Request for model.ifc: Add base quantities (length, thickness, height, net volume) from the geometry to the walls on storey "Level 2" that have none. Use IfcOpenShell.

First a look at what the model holds.

```python
import ifcopenshell
import ifcopenshell.util.element
import ifcopenshell.util.unit

model = ifcopenshell.open("model.ifc")
print(model.schema)
for unit_type in ("LENGTHUNIT", "AREAUNIT", "VOLUMEUNIT"):
    print(unit_type, ifcopenshell.util.unit.calculate_unit_scale(model, unit_type))
storey = next(s for s in model.by_type("IfcBuildingStorey") if s.Name == "Level 2")
walls = [e for e in ifcopenshell.util.element.get_decomposition(storey) if e.is_a("IfcWall")]
for e in sorted(walls, key=lambda e: e.id()):
    print(e.id(), e.is_a(), e.Name, list(ifcopenshell.util.element.get_psets(e, qtos_only=True)), sep=" | ")
```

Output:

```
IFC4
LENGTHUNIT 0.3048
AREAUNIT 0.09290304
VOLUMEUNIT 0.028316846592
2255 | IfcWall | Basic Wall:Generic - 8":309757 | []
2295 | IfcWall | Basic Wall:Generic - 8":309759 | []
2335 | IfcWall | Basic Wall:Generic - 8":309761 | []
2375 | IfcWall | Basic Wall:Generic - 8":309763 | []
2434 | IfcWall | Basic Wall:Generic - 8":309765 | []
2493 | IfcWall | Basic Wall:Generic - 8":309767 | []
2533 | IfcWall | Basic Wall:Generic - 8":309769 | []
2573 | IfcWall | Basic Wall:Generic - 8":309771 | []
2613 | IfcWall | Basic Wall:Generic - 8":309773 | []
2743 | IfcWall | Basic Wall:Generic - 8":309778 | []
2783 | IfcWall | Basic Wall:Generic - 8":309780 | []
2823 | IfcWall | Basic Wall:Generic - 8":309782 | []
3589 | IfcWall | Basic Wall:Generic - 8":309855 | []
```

```python
import ifcopenshell
import ifcopenshell.api.pset
import ifcopenshell.geom
import ifcopenshell.util.element
import ifcopenshell.util.shape
import ifcopenshell.util.unit

model = ifcopenshell.open("model.ifc")
unit_scale = ifcopenshell.util.unit.calculate_unit_scale(model)
volume_scale = ifcopenshell.util.unit.calculate_unit_scale(model, "VOLUMEUNIT")
settings = ifcopenshell.geom.settings()

storey = next(s for s in model.by_type("IfcBuildingStorey") if s.Name == "Level 2")
walls = [e for e in ifcopenshell.util.element.get_decomposition(storey) if e.is_a("IfcWall")]

for e in sorted(walls, key=lambda e: e.id()):
    if ifcopenshell.util.element.get_psets(e, qtos_only=True, should_inherit=False):
        continue
    # Geometry comes back in metres, in the element's own axes.
    shape = ifcopenshell.geom.create_shape(settings, e)
    values = {
        "Length": ifcopenshell.util.shape.get_x(shape.geometry) / unit_scale,
        "Width": ifcopenshell.util.shape.get_y(shape.geometry) / unit_scale,
        "Height": ifcopenshell.util.shape.get_z(shape.geometry) / unit_scale,
        "NetVolume": ifcopenshell.util.shape.get_volume(shape.geometry) / volume_scale,
    }
    qto = ifcopenshell.api.pset.add_qto(model, product=e, name="Qto_WallBaseQuantities")
    ifcopenshell.api.pset.edit_qto(model, qto=qto, properties=values)
    print(e.id(), {k: round(v, 3) for k, v in values.items()})

model.write("model_rev.ifc")
```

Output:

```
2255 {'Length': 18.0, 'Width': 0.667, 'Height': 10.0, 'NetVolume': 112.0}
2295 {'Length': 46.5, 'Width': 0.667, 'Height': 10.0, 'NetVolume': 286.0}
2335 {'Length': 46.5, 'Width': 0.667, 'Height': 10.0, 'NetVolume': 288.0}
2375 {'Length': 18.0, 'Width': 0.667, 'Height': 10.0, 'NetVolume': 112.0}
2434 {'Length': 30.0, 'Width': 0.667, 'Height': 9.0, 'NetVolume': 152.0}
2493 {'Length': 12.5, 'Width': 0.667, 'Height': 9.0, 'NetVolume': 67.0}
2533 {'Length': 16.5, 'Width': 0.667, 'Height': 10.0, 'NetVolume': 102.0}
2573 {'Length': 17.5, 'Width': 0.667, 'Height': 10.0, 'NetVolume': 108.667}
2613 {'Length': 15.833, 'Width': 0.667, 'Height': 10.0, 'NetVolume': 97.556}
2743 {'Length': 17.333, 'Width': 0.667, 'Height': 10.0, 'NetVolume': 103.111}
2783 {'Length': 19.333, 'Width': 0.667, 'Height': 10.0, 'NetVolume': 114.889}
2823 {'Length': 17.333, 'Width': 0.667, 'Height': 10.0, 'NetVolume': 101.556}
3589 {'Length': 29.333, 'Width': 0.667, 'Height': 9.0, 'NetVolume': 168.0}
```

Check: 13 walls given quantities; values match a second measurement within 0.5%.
